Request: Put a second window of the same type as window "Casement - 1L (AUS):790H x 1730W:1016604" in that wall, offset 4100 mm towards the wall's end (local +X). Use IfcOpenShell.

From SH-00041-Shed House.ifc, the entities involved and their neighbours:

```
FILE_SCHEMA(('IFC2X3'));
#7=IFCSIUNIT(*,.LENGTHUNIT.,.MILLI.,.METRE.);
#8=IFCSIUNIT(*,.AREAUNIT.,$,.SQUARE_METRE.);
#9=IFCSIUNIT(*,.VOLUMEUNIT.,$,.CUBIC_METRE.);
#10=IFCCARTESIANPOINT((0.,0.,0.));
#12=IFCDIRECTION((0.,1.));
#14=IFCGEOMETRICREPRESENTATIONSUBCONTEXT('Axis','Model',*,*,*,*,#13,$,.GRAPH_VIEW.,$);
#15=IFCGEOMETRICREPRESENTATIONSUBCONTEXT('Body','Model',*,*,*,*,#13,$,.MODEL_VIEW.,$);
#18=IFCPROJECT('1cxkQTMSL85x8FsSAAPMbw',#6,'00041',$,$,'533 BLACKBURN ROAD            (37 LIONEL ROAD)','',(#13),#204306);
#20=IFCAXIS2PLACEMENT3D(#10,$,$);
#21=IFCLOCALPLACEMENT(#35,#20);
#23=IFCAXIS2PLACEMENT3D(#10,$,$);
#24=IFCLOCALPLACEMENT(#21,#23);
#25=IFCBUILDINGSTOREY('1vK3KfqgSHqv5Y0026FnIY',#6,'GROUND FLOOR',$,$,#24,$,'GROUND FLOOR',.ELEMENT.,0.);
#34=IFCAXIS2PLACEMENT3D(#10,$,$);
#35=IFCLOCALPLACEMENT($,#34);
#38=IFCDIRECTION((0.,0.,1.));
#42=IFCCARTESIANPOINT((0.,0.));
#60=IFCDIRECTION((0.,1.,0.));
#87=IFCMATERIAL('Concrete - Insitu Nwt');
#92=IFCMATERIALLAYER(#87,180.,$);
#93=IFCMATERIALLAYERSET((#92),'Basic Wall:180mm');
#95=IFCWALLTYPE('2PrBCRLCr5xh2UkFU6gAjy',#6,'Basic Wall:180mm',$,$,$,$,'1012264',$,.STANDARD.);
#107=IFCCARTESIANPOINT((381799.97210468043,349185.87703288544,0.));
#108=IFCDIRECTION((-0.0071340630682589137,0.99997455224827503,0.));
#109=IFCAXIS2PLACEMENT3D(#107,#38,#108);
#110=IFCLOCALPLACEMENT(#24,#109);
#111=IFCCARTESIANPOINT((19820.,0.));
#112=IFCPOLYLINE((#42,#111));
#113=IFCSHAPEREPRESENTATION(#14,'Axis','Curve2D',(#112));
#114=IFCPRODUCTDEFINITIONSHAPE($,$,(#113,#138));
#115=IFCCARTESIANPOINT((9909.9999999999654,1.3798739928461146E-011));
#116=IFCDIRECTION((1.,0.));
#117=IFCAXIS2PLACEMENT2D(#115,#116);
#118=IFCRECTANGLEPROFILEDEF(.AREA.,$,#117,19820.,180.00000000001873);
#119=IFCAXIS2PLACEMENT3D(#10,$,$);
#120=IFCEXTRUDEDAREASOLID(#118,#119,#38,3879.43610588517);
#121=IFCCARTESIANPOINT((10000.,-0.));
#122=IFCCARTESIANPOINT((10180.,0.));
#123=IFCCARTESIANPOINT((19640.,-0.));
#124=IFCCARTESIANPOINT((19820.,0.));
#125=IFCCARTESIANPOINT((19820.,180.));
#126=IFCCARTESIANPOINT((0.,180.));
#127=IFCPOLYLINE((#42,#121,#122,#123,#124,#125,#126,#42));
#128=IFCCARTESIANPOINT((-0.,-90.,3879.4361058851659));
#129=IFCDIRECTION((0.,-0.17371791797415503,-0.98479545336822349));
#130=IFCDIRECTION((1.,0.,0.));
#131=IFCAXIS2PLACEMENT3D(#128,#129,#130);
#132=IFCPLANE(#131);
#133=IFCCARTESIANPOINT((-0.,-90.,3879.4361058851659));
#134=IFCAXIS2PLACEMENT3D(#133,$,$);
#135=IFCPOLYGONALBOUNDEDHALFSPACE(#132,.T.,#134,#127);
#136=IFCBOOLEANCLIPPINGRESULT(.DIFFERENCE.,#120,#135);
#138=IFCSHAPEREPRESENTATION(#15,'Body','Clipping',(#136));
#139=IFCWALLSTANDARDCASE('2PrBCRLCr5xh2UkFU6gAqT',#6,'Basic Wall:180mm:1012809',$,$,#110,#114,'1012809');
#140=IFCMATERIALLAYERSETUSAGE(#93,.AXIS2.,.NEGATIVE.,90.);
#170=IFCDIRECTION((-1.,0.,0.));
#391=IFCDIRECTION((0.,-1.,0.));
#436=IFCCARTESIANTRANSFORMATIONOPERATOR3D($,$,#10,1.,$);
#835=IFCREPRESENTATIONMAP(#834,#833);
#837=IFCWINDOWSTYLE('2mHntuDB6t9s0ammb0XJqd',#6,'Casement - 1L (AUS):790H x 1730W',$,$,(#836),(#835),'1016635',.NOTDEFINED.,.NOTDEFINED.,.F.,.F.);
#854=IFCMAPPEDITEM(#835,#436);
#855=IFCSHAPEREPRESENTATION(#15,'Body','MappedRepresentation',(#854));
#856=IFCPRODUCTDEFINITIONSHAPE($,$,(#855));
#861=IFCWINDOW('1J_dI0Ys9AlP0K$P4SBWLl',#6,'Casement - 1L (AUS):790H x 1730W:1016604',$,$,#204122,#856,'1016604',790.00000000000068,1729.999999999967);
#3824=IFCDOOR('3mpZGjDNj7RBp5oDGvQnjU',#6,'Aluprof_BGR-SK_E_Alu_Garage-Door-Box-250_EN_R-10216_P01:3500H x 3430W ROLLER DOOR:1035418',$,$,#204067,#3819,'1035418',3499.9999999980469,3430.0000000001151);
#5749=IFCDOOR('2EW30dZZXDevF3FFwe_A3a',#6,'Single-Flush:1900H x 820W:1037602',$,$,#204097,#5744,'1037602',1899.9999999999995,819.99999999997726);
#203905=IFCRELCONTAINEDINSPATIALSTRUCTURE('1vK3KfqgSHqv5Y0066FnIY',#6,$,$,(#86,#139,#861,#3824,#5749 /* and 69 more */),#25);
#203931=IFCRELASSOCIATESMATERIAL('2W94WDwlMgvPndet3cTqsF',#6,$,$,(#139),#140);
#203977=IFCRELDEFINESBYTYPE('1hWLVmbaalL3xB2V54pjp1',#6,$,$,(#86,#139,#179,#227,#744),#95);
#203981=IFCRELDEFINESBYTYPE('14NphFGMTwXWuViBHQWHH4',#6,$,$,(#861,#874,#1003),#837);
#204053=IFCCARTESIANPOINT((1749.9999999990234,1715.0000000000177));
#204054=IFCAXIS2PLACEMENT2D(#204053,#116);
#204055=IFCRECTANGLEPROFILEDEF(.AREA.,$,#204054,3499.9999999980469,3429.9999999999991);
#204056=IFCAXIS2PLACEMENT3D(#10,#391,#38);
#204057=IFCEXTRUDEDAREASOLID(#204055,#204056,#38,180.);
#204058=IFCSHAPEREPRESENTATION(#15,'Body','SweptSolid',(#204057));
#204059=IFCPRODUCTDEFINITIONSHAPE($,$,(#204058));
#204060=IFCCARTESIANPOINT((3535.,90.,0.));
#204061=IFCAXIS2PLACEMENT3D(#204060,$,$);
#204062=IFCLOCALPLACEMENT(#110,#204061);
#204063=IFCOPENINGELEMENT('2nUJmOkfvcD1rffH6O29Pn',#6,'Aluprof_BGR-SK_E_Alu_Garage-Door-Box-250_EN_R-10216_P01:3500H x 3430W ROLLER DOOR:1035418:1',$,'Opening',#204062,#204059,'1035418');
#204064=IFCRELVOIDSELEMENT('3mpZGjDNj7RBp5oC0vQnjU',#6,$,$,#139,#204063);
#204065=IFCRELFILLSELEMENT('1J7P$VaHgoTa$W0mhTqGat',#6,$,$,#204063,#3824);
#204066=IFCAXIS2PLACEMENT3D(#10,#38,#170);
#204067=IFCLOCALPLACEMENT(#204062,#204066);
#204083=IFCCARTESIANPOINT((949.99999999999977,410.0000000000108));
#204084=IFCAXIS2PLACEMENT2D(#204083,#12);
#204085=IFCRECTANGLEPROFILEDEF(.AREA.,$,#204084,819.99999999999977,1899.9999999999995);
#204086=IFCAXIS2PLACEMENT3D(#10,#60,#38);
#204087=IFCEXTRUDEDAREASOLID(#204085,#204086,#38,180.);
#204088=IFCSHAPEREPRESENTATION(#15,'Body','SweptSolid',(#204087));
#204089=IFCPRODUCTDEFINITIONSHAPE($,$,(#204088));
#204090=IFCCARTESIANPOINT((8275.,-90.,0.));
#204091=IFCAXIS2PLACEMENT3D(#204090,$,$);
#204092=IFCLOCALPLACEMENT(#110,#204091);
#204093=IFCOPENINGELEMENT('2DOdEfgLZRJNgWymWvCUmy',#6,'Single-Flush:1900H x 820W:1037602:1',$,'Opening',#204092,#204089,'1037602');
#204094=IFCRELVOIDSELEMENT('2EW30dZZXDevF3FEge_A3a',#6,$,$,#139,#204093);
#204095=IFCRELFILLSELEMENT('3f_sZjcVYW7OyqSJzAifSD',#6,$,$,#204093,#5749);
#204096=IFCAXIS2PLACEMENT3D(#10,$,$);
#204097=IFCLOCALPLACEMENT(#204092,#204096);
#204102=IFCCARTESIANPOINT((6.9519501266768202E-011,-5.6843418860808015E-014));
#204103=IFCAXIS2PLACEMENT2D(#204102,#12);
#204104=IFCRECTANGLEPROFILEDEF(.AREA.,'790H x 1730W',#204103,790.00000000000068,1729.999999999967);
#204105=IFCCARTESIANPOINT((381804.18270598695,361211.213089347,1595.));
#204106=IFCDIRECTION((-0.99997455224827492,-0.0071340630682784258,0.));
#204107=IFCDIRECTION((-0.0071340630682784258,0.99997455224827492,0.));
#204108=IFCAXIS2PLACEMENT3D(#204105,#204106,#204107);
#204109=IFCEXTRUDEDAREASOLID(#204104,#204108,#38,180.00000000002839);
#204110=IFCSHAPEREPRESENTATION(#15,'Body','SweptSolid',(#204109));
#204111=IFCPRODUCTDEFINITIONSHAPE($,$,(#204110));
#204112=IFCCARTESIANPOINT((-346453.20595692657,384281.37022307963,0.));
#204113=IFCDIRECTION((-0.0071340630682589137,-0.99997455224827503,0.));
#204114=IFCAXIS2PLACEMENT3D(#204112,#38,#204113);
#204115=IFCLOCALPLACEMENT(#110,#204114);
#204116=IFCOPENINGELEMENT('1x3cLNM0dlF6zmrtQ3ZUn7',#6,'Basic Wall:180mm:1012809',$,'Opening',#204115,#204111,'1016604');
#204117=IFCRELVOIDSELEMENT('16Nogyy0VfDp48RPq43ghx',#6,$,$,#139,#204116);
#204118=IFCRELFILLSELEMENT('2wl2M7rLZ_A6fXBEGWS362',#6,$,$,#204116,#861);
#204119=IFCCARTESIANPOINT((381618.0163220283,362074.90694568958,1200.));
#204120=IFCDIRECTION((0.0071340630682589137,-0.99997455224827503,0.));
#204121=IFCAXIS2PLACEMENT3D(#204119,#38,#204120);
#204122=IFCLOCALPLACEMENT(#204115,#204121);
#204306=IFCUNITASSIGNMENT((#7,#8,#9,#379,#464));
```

```python
import ifcopenshell
import ifcopenshell.api.feature
import ifcopenshell.api.geometry
import ifcopenshell.api.root
import ifcopenshell.geom
import ifcopenshell.util.element
import ifcopenshell.util.placement
import ifcopenshell.util.shape
import ifcopenshell.util.unit

model = ifcopenshell.open("SH-00041-Shed House.ifc")
unit_scale = ifcopenshell.util.unit.calculate_unit_scale(model)
settings = ifcopenshell.geom.settings()


def volume(element):
    """Net volume in cubic metres, openings subtracted."""
    shape = ifcopenshell.geom.create_shape(settings, element)
    return ifcopenshell.util.shape.get_volume(shape.geometry)


def reuse_history(source, copy):
    """copy_class also copies each property set's owner history, people and application; keep the originals."""
    for rel in copy.IsDefinedBy:
        if rel.is_a("IfcRelDefinesByProperties") and (history := rel.RelatingPropertyDefinition.OwnerHistory):
            rel.RelatingPropertyDefinition.OwnerHistory = source.OwnerHistory
            ifcopenshell.util.element.remove_deep2(model, history)


window = model.by_id(861)
opening = window.FillsVoids[0].RelatingOpeningElement
wall = opening.VoidsElements[0].RelatingBuildingElement
before = volume(wall)
shift = ifcopenshell.util.placement.get_local_placement(wall.ObjectPlacement)[:3, 0] * 4.1 / unit_scale

# copy_class copies the void relationship, type, container and properties, but no geometry.
new_opening = ifcopenshell.api.root.copy_class(model, product=opening)
new_opening.Representation = ifcopenshell.util.element.copy_deep(
    model, opening.Representation, exclude=["IfcGeometricRepresentationContext", "IfcRepresentationMap"]
)
new_opening.Name = "Basic Wall:180mm"
new_opening.Tag = None
new_window = ifcopenshell.api.root.copy_class(model, product=window)
new_window.Representation = ifcopenshell.util.element.copy_deep(
    model, window.Representation, exclude=["IfcGeometricRepresentationContext", "IfcRepresentationMap"]
)
new_window.Name = "Casement - 1L (AUS):790H x 1730W"
new_window.Tag = None
reuse_history(window, new_window)
fills = ifcopenshell.api.feature.add_filling(model, opening=new_opening, element=new_window)
fills.OwnerHistory = new_window.OwnerHistory  # required in IFC2X3

for old, new in ((opening, new_opening), (window, new_window)):
    matrix = ifcopenshell.util.placement.get_local_placement(old.ObjectPlacement)
    matrix[:3, 3] += shift
    ifcopenshell.api.geometry.edit_object_placement(model, product=new, matrix=matrix, is_si=False)

after = volume(wall)

print(f"wall volume {before:.3f} -> {after:.3f} m3")

model.write("SH-00041-Shed House_v2.ifc")
```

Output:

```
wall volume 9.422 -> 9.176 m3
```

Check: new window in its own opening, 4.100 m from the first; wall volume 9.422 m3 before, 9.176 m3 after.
